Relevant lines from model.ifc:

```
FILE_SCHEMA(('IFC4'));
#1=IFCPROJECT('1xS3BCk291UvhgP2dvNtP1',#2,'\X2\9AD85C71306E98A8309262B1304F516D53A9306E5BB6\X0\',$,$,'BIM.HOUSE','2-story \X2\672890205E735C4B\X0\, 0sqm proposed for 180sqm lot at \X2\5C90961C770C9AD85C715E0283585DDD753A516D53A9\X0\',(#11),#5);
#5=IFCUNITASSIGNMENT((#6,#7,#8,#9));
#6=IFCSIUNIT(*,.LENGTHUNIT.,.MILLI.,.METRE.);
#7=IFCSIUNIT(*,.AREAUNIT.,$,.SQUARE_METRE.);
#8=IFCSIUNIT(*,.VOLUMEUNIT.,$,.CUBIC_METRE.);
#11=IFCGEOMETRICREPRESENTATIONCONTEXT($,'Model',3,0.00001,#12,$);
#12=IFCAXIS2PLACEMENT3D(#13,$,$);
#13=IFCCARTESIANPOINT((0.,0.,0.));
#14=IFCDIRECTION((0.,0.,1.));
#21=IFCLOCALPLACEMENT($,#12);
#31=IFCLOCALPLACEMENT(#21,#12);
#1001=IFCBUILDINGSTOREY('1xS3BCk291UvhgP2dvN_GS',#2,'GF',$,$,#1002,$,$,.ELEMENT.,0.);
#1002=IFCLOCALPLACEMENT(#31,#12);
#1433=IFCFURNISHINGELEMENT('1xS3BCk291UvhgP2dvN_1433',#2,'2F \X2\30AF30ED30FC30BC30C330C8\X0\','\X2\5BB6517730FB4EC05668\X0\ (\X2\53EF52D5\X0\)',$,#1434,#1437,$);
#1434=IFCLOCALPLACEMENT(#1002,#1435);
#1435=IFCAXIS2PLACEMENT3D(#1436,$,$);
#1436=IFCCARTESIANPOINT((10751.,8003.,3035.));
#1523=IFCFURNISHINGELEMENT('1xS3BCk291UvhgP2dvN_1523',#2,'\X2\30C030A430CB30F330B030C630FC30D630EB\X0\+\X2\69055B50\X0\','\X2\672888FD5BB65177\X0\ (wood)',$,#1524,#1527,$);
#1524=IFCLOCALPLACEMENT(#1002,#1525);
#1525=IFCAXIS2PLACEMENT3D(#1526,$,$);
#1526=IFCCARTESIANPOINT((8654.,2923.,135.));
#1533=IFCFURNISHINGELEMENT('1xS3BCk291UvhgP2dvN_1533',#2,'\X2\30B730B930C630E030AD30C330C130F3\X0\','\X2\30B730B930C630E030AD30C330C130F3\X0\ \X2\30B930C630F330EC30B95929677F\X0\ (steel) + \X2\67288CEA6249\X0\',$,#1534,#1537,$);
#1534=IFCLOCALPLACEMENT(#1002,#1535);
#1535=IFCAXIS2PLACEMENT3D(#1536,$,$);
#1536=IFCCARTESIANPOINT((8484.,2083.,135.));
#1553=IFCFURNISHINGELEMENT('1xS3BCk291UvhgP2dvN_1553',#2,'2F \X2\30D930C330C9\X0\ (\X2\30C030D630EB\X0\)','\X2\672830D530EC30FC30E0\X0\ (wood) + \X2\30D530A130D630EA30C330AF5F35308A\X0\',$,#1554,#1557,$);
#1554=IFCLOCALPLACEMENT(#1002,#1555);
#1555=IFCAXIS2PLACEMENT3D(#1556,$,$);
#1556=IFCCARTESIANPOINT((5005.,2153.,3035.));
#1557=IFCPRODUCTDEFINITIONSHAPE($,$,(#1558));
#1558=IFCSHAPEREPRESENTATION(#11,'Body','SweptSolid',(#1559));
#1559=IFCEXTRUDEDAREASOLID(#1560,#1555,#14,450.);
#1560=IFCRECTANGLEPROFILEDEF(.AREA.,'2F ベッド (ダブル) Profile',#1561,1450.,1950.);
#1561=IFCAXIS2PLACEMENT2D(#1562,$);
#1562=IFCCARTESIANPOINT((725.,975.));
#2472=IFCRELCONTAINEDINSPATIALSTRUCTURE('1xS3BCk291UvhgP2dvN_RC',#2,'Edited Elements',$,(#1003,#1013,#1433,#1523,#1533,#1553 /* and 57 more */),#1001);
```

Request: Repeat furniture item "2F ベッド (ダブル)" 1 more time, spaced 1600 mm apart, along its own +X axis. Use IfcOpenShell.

```python
import ifcopenshell
import ifcopenshell.api.geometry
import ifcopenshell.api.root
import ifcopenshell.util.element
import ifcopenshell.util.placement
import ifcopenshell.util.unit

model = ifcopenshell.open("model.ifc")
unit_scale = ifcopenshell.util.unit.calculate_unit_scale(model)


def reuse_history(source, copy):
    """copy_class also copies each property set's owner history, people and application; keep the originals."""
    for rel in copy.IsDefinedBy:
        if rel.is_a("IfcRelDefinesByProperties") and (history := rel.RelatingPropertyDefinition.OwnerHistory):
            rel.RelatingPropertyDefinition.OwnerHistory = source.OwnerHistory
            ifcopenshell.util.element.remove_deep2(model, history)


source = model.by_guid("1xS3BCk291UvhgP2dvN_1553")
base = ifcopenshell.util.placement.get_local_placement(source.ObjectPlacement)
step = base[:3, 0] * 1.6 / unit_scale

for i in range(1, 2):
    copy = ifcopenshell.api.root.copy_class(model, product=source)
    copy.Representation = ifcopenshell.util.element.copy_deep(
        model, source.Representation, exclude=["IfcGeometricRepresentationContext", "IfcRepresentationMap"]
    )
    reuse_history(source, copy)
    matrix = base.copy()
    matrix[:3, 3] += i * step
    print("added at", matrix[:3, 3].round(3) + 0.0)
    ifcopenshell.api.geometry.edit_object_placement(model, product=copy, matrix=matrix, is_si=False)

model.write("model_rev.ifc")
```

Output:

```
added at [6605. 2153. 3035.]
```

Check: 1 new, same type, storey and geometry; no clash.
